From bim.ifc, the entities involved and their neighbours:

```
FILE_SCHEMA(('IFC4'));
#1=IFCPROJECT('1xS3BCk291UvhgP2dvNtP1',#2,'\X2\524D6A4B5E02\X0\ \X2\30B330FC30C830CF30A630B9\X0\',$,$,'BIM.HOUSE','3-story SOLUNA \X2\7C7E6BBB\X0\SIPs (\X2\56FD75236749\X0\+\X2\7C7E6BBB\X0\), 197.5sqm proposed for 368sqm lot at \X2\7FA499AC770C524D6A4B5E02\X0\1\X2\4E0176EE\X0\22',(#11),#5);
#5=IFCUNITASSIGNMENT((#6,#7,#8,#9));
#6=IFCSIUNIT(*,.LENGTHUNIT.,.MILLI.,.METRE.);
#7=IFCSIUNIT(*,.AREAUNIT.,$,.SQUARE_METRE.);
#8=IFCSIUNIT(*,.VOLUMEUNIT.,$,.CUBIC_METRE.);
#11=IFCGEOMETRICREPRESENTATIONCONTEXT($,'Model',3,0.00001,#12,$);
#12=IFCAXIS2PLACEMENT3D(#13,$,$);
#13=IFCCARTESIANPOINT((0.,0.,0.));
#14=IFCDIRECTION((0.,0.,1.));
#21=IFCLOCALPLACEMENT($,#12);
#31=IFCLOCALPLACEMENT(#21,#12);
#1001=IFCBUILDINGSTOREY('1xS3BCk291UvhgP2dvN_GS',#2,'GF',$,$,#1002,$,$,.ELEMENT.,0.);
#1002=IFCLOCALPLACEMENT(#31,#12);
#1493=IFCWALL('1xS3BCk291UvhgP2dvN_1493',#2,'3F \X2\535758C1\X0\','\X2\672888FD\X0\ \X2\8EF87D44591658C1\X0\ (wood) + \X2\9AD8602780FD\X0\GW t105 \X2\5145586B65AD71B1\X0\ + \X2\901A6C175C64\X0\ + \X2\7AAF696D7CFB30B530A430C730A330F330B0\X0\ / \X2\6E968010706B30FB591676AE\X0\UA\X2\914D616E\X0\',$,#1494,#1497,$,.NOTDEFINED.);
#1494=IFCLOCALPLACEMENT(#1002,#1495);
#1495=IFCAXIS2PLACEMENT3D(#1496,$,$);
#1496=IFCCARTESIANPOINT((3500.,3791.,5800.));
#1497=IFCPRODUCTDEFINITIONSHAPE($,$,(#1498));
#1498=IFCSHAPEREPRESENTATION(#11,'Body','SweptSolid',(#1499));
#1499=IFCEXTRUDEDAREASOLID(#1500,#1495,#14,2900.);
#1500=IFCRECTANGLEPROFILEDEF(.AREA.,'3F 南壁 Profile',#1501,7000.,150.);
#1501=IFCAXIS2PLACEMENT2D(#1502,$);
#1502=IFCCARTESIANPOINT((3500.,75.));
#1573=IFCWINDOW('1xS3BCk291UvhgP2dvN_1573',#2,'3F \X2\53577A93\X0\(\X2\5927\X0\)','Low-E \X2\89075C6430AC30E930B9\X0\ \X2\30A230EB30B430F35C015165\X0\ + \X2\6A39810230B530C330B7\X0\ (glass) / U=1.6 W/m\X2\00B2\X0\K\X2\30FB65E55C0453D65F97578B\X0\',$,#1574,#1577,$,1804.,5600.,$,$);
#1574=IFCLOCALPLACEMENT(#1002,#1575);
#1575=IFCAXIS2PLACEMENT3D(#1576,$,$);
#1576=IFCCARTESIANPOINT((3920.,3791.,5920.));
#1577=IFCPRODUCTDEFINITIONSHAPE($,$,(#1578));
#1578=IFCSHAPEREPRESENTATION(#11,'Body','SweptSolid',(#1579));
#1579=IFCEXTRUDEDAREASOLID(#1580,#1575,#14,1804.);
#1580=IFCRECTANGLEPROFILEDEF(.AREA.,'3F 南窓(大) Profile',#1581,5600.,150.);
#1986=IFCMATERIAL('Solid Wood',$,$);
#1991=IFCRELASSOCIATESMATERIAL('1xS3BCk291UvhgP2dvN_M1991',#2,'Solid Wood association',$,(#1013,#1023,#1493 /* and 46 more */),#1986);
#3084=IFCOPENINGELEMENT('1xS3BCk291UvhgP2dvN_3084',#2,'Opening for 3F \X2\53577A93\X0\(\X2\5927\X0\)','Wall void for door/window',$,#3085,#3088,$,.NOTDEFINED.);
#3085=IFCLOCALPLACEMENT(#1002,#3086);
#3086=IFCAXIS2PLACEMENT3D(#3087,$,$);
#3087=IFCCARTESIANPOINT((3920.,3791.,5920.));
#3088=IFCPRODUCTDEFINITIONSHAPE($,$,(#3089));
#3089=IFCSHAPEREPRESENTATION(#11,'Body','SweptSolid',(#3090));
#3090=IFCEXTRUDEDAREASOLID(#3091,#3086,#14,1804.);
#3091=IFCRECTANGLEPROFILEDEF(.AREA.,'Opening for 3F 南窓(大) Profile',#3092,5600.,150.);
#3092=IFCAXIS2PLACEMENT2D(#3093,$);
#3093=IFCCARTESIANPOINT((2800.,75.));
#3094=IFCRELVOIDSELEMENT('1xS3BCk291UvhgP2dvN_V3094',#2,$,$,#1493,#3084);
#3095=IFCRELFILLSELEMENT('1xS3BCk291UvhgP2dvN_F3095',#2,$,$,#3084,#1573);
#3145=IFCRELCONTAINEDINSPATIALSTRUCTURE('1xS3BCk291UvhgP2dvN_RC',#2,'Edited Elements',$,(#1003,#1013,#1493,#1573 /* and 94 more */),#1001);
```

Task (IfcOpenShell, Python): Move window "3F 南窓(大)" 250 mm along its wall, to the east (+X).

```python
import ifcopenshell
import ifcopenshell.api.geometry
import ifcopenshell.util.placement

model = ifcopenshell.open("bim.ifc")

window = model.by_guid("1xS3BCk291UvhgP2dvN_1573")
opening = window.FillsVoids[0].RelatingOpeningElement
wall = opening.VoidsElements[0].RelatingBuildingElement

wall_matrix = ifcopenshell.util.placement.get_local_placement(wall.ObjectPlacement)
shift = wall_matrix[:3, 0] * 250.0
before = ifcopenshell.util.placement.get_local_placement(window.ObjectPlacement)[:3, 3].copy()

# The window is not placed relative to its opening, so move both.
for product in (opening, window):
    matrix = ifcopenshell.util.placement.get_local_placement(product.ObjectPlacement)
    matrix[:3, 3] += shift
    ifcopenshell.api.geometry.edit_object_placement(model, product=product, matrix=matrix, is_si=False)

after = ifcopenshell.util.placement.get_local_placement(window.ObjectPlacement)[:3, 3]
print("window moved by", (after - before).round(3) + 0.0)

model.write("bim_rev.ifc")
```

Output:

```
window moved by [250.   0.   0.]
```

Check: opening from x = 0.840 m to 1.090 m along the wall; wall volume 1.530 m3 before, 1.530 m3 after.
